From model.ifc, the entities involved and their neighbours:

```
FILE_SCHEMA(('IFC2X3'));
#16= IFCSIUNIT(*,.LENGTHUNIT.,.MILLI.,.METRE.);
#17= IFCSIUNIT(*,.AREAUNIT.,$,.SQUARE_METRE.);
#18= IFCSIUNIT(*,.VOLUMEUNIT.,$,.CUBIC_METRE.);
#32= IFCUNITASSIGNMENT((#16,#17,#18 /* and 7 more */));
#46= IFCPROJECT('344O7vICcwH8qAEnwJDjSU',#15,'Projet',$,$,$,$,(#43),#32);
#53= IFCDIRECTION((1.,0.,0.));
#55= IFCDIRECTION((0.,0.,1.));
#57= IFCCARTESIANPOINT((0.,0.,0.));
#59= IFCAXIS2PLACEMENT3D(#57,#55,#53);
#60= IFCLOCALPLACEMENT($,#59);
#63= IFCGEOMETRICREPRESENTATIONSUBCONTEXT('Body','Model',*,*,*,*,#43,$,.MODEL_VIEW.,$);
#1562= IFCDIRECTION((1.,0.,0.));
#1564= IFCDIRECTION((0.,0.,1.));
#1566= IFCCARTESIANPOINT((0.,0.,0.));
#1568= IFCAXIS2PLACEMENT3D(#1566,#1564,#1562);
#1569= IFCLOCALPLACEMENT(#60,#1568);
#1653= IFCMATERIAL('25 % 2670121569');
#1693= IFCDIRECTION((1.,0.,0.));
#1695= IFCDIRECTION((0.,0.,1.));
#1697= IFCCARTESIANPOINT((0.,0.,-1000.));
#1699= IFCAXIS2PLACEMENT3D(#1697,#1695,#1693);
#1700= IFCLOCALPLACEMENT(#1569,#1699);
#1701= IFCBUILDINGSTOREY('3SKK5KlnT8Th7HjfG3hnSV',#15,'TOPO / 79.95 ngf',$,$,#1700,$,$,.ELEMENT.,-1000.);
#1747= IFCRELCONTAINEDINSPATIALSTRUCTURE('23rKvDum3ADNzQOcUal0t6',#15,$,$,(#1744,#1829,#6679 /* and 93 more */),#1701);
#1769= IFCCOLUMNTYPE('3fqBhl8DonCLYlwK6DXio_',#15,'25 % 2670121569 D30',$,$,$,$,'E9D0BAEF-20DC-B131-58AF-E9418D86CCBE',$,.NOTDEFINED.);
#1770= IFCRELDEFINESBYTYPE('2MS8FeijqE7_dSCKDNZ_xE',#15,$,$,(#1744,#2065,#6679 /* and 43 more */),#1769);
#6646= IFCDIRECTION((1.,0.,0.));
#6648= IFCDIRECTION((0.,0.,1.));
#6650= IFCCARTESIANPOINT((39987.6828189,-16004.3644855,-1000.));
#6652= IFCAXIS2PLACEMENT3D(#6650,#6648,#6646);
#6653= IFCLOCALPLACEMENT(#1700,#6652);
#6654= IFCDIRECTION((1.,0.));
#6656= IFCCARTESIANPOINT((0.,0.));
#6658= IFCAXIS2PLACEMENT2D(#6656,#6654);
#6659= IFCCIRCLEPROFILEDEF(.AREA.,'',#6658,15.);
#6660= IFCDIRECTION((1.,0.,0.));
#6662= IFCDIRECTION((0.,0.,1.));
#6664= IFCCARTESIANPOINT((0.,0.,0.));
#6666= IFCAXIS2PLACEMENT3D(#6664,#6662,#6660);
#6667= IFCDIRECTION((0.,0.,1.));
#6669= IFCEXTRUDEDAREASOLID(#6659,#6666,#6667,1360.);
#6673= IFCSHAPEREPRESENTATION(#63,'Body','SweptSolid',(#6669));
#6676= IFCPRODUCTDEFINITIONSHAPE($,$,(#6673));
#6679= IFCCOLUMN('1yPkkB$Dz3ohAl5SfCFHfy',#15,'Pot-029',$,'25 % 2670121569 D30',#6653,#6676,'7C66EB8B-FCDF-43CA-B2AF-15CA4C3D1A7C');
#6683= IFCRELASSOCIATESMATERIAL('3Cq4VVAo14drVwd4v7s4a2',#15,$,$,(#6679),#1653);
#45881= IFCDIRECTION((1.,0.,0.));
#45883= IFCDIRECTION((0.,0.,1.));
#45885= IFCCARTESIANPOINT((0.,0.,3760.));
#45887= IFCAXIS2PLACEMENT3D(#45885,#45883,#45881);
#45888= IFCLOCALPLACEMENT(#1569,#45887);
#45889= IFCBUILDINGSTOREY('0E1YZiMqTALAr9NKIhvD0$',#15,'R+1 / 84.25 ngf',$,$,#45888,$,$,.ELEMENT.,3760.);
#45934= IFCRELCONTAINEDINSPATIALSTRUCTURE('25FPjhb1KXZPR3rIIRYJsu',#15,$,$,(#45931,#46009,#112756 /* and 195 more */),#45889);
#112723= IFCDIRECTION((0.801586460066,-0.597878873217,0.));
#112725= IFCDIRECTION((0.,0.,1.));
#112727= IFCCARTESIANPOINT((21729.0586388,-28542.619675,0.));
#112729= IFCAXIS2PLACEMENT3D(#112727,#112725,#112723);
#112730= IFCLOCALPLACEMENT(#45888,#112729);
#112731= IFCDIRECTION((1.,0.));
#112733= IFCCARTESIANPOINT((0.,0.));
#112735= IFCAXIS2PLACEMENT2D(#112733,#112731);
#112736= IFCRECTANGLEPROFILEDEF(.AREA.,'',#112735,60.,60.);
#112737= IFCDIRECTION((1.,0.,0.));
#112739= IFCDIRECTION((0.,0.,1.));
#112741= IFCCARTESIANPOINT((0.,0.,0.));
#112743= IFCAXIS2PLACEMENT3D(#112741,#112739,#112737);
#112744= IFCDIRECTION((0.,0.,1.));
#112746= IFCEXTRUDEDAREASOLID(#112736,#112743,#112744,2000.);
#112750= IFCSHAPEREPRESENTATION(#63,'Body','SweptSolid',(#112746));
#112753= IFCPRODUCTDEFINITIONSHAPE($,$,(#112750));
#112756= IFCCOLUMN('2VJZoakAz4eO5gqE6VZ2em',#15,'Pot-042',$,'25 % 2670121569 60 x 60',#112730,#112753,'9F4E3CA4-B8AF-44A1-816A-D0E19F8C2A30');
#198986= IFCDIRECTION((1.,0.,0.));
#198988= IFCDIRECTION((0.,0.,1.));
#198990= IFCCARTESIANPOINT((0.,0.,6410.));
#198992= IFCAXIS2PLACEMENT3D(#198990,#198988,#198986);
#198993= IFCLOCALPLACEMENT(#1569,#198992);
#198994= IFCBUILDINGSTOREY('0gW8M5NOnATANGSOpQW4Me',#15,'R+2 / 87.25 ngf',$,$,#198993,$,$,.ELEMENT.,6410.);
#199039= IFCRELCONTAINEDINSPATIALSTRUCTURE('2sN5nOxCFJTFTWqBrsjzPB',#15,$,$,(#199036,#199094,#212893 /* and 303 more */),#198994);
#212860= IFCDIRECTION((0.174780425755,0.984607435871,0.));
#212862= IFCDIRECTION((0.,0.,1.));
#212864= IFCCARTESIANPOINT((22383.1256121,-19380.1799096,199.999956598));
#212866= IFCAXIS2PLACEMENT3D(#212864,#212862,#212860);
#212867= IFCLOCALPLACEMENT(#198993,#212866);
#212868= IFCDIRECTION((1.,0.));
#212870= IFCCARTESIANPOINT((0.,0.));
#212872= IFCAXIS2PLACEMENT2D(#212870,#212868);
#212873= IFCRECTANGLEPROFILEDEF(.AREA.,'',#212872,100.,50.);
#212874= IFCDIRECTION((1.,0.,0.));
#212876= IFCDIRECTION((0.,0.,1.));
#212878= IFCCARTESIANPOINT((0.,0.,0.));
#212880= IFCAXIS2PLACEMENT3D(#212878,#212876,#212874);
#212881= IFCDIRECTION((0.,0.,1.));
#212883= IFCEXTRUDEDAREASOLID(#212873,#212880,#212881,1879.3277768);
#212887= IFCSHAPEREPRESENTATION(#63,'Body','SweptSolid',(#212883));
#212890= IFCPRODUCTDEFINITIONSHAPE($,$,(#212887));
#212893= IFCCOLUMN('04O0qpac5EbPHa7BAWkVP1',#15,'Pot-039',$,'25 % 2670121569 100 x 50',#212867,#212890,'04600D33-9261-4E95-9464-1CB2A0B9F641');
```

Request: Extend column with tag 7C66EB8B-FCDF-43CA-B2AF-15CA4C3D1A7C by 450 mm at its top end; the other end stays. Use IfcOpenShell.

```python
import ifcopenshell
import ifcopenshell.util.representation
import ifcopenshell.util.unit

model = ifcopenshell.open("model.ifc")
unit_scale = ifcopenshell.util.unit.calculate_unit_scale(model)

member = model.by_guid("1yPkkB$Dz3ohAl5SfCFHfy")
change = 0.45 / unit_scale

# The extrusion runs towards the end named, so only its depth changes.
body = ifcopenshell.util.representation.get_representation(member, "Model", "Body")
solid = body.Items[0]
old_length = solid.Depth
solid.Depth += change

print(f"length {old_length:g} -> {solid.Depth:g}")

model.write("model-out.ifc")
```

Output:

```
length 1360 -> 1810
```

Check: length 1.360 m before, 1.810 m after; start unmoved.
